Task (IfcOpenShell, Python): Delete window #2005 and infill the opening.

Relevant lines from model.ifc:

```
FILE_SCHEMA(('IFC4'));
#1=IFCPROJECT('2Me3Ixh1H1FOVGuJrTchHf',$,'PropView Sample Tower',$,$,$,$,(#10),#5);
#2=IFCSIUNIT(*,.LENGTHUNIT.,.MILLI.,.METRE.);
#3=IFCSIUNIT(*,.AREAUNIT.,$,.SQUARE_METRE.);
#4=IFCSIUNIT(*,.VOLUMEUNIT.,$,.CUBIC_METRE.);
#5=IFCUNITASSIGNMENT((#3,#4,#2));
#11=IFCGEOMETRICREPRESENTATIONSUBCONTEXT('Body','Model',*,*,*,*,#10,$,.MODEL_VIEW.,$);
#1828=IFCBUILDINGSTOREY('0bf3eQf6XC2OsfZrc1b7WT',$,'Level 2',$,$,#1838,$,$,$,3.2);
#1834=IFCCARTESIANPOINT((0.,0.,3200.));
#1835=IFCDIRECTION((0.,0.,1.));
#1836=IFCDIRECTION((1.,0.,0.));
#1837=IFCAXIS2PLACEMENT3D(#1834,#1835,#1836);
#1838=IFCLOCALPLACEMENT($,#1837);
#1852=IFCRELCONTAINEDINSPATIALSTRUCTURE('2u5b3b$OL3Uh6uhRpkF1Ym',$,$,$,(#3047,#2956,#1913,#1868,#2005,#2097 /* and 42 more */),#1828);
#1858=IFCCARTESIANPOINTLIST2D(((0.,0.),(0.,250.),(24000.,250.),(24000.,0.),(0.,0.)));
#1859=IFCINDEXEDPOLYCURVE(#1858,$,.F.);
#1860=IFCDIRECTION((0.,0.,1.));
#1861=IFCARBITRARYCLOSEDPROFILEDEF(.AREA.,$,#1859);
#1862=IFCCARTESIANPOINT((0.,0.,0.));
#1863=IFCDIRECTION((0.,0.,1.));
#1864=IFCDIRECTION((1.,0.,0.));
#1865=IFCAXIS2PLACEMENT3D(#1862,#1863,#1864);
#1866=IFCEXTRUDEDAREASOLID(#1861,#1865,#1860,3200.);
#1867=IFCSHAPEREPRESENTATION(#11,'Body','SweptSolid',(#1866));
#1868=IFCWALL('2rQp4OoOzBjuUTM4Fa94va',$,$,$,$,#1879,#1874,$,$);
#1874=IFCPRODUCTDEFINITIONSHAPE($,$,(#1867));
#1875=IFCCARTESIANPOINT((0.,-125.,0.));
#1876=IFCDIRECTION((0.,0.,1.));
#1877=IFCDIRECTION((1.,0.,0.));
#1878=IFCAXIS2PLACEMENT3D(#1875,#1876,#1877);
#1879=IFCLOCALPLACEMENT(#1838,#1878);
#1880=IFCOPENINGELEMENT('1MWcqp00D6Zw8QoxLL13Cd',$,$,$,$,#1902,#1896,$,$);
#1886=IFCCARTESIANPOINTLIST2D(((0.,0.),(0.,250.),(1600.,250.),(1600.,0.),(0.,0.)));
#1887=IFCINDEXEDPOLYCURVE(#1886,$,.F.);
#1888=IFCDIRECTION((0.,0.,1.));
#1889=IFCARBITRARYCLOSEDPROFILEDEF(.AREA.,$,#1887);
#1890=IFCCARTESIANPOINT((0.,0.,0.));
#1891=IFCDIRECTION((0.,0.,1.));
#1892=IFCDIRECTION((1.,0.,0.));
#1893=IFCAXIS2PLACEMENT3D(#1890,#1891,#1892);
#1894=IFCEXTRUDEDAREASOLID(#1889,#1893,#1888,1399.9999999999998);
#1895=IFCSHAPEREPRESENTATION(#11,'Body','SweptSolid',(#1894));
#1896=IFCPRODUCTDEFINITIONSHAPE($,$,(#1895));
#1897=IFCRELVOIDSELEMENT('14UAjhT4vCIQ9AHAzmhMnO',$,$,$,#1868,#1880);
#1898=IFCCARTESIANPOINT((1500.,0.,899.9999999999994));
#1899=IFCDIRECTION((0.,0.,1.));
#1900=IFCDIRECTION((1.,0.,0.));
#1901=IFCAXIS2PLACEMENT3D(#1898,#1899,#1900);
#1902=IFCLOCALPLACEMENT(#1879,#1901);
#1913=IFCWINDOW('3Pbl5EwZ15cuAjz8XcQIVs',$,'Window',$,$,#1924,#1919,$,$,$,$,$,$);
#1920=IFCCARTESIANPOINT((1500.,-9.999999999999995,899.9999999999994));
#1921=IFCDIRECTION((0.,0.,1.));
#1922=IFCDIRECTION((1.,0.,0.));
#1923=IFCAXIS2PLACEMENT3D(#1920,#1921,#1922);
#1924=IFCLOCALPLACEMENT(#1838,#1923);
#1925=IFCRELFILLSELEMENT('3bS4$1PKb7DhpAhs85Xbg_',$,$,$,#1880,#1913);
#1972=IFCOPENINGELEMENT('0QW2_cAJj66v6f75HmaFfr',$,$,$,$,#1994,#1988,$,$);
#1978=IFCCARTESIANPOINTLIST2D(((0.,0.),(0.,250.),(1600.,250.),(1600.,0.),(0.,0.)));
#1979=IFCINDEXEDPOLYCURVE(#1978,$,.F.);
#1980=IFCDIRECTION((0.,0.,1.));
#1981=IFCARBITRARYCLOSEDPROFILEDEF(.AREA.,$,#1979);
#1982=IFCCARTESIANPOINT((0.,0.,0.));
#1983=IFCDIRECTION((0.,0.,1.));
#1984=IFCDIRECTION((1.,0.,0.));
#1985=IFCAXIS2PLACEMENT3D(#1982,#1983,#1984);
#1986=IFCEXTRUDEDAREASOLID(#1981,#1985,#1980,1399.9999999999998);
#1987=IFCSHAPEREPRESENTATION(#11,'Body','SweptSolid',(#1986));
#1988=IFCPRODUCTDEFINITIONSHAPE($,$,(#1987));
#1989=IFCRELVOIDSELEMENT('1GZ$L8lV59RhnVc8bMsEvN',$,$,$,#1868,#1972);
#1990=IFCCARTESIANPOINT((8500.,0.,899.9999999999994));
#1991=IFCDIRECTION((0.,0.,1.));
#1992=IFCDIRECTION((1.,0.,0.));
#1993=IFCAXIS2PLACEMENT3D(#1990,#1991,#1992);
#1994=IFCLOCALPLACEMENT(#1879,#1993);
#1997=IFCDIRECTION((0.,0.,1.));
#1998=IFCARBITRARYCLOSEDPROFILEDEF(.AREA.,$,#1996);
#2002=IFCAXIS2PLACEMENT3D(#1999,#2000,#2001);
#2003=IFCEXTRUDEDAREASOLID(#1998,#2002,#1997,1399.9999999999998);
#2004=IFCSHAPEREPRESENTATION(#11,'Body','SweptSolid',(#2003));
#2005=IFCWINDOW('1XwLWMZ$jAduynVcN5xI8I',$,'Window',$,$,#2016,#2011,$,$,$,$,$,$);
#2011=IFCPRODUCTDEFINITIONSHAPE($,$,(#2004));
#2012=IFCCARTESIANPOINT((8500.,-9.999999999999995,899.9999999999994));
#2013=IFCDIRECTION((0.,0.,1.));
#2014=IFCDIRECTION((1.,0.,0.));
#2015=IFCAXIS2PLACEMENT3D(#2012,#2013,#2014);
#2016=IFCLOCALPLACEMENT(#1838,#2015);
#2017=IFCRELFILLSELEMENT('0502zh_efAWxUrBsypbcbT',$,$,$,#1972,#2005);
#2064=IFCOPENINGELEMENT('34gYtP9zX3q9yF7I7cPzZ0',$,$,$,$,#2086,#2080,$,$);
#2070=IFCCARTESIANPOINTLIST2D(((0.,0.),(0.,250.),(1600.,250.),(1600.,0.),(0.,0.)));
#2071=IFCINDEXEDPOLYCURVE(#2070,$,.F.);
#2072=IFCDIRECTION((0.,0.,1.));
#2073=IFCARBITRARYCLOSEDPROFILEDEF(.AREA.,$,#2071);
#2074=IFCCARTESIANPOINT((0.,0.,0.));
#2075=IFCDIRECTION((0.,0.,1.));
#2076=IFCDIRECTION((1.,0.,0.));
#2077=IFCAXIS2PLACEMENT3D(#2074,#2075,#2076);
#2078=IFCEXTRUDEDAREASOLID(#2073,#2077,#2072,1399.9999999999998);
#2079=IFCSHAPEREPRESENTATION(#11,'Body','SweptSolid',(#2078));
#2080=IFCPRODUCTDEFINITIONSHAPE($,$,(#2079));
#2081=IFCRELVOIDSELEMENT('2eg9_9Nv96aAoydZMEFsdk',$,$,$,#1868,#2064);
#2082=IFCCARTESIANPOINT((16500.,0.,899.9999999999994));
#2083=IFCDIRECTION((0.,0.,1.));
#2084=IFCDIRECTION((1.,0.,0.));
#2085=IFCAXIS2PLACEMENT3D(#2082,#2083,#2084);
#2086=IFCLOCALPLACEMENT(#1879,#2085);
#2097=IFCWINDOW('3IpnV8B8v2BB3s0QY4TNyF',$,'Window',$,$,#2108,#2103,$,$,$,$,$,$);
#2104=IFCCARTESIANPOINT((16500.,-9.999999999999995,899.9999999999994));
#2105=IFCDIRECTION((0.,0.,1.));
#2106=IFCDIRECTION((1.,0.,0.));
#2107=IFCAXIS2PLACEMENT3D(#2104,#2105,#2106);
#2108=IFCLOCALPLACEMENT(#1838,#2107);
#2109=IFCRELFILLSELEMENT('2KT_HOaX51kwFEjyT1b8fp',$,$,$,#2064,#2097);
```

```python
import ifcopenshell
import ifcopenshell.api.feature
import ifcopenshell.api.root
import ifcopenshell.geom
import ifcopenshell.util.shape

model = ifcopenshell.open("model.ifc")
settings = ifcopenshell.geom.settings()


def volume(element):
    """Net volume in cubic metres, openings subtracted."""
    shape = ifcopenshell.geom.create_shape(settings, element)
    return ifcopenshell.util.shape.get_volume(shape.geometry)


window = model.by_id(2005)
opening = window.FillsVoids[0].RelatingOpeningElement
wall = opening.VoidsElements[0].RelatingBuildingElement
before = volume(wall)

ifcopenshell.api.root.remove_product(model, product=window)
ifcopenshell.api.feature.remove_feature(model, feature=opening)

after = volume(wall)

print(f"wall volume {before:.3f} -> {after:.3f} m3")

model.write("model_rev.ifc")
```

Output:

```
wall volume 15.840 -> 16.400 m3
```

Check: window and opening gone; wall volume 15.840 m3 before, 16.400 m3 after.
